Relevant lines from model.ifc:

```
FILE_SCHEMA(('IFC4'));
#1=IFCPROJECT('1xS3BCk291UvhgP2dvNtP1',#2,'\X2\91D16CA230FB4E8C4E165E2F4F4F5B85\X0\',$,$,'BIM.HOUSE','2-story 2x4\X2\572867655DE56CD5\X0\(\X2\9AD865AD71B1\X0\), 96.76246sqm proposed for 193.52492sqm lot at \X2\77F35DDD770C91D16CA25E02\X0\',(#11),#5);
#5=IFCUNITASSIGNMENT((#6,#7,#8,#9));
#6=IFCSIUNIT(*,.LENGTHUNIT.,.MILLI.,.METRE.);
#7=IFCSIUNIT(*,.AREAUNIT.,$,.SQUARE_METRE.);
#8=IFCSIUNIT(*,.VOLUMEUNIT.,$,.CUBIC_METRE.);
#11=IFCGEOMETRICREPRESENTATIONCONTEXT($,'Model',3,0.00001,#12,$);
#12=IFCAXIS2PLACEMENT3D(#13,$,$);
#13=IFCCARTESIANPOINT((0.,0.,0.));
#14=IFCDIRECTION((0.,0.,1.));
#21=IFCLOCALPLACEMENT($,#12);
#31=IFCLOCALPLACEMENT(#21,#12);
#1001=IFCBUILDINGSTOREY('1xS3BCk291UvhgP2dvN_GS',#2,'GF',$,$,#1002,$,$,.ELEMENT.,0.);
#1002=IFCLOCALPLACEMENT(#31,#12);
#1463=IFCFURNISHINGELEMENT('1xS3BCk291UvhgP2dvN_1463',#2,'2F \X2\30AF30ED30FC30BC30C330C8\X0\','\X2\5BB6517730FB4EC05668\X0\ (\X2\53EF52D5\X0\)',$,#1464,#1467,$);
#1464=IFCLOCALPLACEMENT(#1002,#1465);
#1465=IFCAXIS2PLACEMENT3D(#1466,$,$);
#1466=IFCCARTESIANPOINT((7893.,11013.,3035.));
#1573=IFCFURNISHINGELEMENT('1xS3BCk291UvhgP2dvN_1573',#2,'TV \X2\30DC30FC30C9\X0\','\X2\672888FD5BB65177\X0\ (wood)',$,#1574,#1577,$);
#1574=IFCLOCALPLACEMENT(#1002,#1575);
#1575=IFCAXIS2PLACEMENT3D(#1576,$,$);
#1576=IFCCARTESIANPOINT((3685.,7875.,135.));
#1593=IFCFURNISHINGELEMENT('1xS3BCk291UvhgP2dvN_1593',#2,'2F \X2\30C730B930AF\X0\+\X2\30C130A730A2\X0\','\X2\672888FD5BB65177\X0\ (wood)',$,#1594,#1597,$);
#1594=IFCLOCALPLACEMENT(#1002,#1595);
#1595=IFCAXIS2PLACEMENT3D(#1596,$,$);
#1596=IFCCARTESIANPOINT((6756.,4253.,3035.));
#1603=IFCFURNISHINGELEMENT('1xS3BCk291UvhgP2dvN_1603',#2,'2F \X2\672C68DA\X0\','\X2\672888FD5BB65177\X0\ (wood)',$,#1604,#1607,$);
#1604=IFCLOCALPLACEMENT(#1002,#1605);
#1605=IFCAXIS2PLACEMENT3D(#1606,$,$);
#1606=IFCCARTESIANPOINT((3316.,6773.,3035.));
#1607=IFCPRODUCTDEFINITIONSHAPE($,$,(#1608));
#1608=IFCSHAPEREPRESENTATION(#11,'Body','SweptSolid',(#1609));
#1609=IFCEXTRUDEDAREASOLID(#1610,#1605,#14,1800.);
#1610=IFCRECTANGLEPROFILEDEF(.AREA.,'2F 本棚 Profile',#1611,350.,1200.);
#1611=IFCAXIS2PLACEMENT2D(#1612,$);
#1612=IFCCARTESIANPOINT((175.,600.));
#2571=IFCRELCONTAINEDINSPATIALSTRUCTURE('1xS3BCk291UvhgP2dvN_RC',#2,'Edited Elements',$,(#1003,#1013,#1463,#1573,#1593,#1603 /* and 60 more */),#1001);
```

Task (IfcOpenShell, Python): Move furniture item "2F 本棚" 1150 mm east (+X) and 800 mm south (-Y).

```python
import ifcopenshell
import ifcopenshell.api.geometry
import ifcopenshell.util.placement
import ifcopenshell.util.unit

model = ifcopenshell.open("model.ifc")
unit_scale = ifcopenshell.util.unit.calculate_unit_scale(model)

item = model.by_id(1603)
matrix = ifcopenshell.util.placement.get_local_placement(item.ObjectPlacement)
matrix[0, 3] += 1.15 / unit_scale
matrix[1, 3] -= 0.8 / unit_scale
ifcopenshell.api.geometry.edit_object_placement(model, product=item, matrix=matrix, is_si=False)

print(ifcopenshell.util.placement.get_local_placement(item.ObjectPlacement).round(3) + 0.0)

model.write("model_updated.ifc")
```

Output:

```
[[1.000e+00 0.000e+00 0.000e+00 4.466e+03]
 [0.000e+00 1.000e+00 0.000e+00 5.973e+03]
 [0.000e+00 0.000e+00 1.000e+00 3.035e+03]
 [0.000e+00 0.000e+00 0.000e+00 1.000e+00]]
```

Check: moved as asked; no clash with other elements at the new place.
